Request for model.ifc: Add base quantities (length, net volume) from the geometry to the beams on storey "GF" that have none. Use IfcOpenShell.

First a look at what the model holds.

```python
import ifcopenshell
import ifcopenshell.util.element
import ifcopenshell.util.unit

model = ifcopenshell.open("model.ifc")
print(model.schema)
for unit_type in ("LENGTHUNIT", "AREAUNIT", "VOLUMEUNIT"):
    print(unit_type, ifcopenshell.util.unit.calculate_unit_scale(model, unit_type))
storey = next(s for s in model.by_type("IfcBuildingStorey") if s.Name == "GF")
beams = [e for e in ifcopenshell.util.element.get_decomposition(storey) if e.is_a("IfcBeam")]
for e in sorted(beams, key=lambda e: e.id()):
    print(e.id(), e.is_a(), e.Name, list(ifcopenshell.util.element.get_psets(e, qtos_only=True)), sep=" | ")
```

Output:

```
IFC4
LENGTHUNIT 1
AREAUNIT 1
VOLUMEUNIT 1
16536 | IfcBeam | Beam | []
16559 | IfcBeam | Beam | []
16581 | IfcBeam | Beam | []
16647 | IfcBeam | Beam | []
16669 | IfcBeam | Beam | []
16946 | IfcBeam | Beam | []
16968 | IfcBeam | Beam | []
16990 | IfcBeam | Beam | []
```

```python
import ifcopenshell
import ifcopenshell.api.pset
import ifcopenshell.geom
import ifcopenshell.util.element
import ifcopenshell.util.shape
import ifcopenshell.util.unit

model = ifcopenshell.open("model.ifc")
unit_scale = ifcopenshell.util.unit.calculate_unit_scale(model)
volume_scale = ifcopenshell.util.unit.calculate_unit_scale(model, "VOLUMEUNIT")
settings = ifcopenshell.geom.settings()

storey = next(s for s in model.by_type("IfcBuildingStorey") if s.Name == "GF")
beams = [e for e in ifcopenshell.util.element.get_decomposition(storey) if e.is_a("IfcBeam")]

for e in sorted(beams, key=lambda e: e.id()):
    if ifcopenshell.util.element.get_psets(e, qtos_only=True, should_inherit=False):
        continue
    # Geometry comes back in metres, in the element's own axes.
    shape = ifcopenshell.geom.create_shape(settings, e)
    values = {
        "Length": ifcopenshell.util.shape.get_max_xyz(shape.geometry) / unit_scale,
        "NetVolume": ifcopenshell.util.shape.get_volume(shape.geometry) / volume_scale,
    }
    qto = ifcopenshell.api.pset.add_qto(model, product=e, name="Qto_BeamBaseQuantities")
    ifcopenshell.api.pset.edit_qto(model, qto=qto, properties=values)
    print(e.id(), {k: round(v, 3) for k, v in values.items()})

model.write("model_rev.ifc")
```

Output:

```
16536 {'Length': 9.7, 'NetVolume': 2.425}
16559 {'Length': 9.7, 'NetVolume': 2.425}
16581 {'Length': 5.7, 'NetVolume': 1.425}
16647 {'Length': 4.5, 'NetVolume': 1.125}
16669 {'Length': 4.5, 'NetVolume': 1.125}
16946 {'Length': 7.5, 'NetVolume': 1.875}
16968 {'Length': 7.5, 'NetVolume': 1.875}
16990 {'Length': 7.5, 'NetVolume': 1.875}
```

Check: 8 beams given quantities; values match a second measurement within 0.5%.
